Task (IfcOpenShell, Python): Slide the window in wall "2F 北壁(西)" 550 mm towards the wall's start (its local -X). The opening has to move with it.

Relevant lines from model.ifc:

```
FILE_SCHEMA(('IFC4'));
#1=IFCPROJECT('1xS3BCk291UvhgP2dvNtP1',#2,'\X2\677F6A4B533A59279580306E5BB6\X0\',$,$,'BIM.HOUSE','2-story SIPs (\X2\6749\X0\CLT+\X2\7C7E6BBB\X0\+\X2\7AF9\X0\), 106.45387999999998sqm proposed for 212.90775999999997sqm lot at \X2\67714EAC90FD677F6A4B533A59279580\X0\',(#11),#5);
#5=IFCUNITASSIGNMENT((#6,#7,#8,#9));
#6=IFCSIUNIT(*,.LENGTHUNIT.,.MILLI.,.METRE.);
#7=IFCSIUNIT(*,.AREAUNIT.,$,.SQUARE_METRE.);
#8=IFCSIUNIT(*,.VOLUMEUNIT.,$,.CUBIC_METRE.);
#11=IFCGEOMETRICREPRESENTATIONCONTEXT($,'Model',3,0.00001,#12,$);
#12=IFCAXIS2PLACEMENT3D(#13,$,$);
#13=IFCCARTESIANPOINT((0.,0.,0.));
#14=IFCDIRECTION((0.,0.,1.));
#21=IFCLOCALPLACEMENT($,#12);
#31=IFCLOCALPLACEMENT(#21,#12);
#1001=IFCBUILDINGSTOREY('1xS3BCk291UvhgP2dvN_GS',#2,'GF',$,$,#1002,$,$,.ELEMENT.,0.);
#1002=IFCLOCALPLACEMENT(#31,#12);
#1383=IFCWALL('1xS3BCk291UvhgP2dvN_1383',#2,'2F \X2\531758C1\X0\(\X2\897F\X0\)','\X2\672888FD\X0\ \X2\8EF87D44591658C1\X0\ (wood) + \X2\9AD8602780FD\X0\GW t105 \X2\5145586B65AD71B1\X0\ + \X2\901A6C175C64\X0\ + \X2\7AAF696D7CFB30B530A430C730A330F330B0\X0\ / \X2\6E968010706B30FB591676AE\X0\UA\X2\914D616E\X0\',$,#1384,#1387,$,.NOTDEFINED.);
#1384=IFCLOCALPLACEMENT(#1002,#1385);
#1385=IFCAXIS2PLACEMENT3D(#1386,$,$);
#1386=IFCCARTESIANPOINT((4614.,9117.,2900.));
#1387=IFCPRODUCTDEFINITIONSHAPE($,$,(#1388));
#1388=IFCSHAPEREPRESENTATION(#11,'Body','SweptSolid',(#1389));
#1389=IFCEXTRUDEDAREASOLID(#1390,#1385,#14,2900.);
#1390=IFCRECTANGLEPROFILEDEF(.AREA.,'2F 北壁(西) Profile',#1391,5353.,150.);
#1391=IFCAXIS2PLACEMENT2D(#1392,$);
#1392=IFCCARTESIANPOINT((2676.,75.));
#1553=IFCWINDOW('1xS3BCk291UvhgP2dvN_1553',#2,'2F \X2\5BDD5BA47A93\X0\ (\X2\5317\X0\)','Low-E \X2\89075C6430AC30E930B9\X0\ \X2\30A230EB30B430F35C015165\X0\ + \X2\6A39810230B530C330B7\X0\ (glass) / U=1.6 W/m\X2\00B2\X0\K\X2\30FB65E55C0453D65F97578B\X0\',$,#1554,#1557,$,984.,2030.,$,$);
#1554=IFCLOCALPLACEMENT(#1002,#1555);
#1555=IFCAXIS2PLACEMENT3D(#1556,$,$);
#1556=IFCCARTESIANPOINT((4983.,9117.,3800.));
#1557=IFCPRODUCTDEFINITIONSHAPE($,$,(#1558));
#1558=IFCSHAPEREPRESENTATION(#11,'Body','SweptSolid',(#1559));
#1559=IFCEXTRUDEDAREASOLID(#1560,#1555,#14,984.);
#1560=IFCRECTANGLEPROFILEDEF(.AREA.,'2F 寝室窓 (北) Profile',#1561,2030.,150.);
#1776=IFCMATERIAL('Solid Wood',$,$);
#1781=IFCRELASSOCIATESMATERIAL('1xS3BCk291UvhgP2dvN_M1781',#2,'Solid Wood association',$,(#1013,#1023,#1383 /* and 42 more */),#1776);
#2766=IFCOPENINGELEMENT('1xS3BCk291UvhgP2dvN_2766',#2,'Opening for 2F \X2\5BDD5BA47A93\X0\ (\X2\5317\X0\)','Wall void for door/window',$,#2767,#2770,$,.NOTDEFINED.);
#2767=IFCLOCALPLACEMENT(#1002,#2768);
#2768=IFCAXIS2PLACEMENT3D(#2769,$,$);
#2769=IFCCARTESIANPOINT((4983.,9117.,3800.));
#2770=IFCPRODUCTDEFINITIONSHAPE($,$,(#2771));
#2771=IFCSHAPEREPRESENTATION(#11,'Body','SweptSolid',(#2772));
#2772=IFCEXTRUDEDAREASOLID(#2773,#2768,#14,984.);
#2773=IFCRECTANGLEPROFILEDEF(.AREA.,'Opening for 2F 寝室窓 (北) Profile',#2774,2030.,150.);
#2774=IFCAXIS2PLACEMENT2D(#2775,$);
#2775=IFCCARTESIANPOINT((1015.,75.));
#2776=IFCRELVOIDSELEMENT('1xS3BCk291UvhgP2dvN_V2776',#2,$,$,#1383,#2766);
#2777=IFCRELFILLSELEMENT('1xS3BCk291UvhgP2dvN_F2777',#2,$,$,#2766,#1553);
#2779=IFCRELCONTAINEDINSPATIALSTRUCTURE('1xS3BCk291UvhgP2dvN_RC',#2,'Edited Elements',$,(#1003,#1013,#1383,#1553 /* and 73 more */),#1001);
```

```python
import ifcopenshell
import ifcopenshell.api.geometry
import ifcopenshell.util.placement

model = ifcopenshell.open("model.ifc")

window = model.by_guid("1xS3BCk291UvhgP2dvN_1553")
opening = window.FillsVoids[0].RelatingOpeningElement
wall = opening.VoidsElements[0].RelatingBuildingElement

wall_matrix = ifcopenshell.util.placement.get_local_placement(wall.ObjectPlacement)
shift = wall_matrix[:3, 0] * -550.0
before = ifcopenshell.util.placement.get_local_placement(window.ObjectPlacement)[:3, 3].copy()

# The window is not placed relative to its opening, so move both.
for product in (opening, window):
    matrix = ifcopenshell.util.placement.get_local_placement(product.ObjectPlacement)
    matrix[:3, 3] += shift
    ifcopenshell.api.geometry.edit_object_placement(model, product=product, matrix=matrix, is_si=False)

after = ifcopenshell.util.placement.get_local_placement(window.ObjectPlacement)[:3, 3]
print("window moved by", (after - before).round(3) + 0.0)

model.write("model_edited.ifc")
```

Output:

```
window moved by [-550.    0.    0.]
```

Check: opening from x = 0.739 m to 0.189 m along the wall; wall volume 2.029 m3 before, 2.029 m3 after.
